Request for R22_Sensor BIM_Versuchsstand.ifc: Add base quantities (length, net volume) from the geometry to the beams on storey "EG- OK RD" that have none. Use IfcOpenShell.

First a look at what the model holds.

```python
import ifcopenshell
import ifcopenshell.util.element
import ifcopenshell.util.unit

model = ifcopenshell.open("R22_Sensor BIM_Versuchsstand.ifc")
print(model.schema)
for unit_type in ("LENGTHUNIT", "AREAUNIT", "VOLUMEUNIT"):
    print(unit_type, ifcopenshell.util.unit.calculate_unit_scale(model, unit_type))
storey = next(s for s in model.by_type("IfcBuildingStorey") if s.Name == "EG- OK RD")
beams = [e for e in ifcopenshell.util.element.get_decomposition(storey) if e.is_a("IfcBeam")]
for e in sorted(beams, key=lambda e: e.id()):
    print(e.id(), e.is_a(), e.Name, list(ifcopenshell.util.element.get_psets(e, qtos_only=True)), sep=" | ")
```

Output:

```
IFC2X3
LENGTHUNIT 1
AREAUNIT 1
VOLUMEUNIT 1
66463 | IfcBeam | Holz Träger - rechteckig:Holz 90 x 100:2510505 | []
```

```python
import ifcopenshell
import ifcopenshell.api.pset
import ifcopenshell.geom
import ifcopenshell.util.element
import ifcopenshell.util.shape
import ifcopenshell.util.unit

model = ifcopenshell.open("R22_Sensor BIM_Versuchsstand.ifc")
unit_scale = ifcopenshell.util.unit.calculate_unit_scale(model)
volume_scale = ifcopenshell.util.unit.calculate_unit_scale(model, "VOLUMEUNIT")
settings = ifcopenshell.geom.settings()

storey = next(s for s in model.by_type("IfcBuildingStorey") if s.Name == "EG- OK RD")
beams = [e for e in ifcopenshell.util.element.get_decomposition(storey) if e.is_a("IfcBeam")]

for e in sorted(beams, key=lambda e: e.id()):
    if ifcopenshell.util.element.get_psets(e, qtos_only=True, should_inherit=False):
        continue
    # Geometry comes back in metres, in the element's own axes.
    shape = ifcopenshell.geom.create_shape(settings, e)
    values = {
        "Length": ifcopenshell.util.shape.get_max_xyz(shape.geometry) / unit_scale,
        "NetVolume": ifcopenshell.util.shape.get_volume(shape.geometry) / volume_scale,
    }
    qto = ifcopenshell.api.pset.add_qto(model, product=e, name="BaseQuantities")
    ifcopenshell.api.pset.edit_qto(model, qto=qto, properties=values)
    print(e.id(), {k: round(v, 3) for k, v in values.items()})

model.write("R22_Sensor BIM_Versuchsstand-out.ifc")
```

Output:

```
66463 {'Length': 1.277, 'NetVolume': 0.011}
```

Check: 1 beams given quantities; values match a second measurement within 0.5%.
